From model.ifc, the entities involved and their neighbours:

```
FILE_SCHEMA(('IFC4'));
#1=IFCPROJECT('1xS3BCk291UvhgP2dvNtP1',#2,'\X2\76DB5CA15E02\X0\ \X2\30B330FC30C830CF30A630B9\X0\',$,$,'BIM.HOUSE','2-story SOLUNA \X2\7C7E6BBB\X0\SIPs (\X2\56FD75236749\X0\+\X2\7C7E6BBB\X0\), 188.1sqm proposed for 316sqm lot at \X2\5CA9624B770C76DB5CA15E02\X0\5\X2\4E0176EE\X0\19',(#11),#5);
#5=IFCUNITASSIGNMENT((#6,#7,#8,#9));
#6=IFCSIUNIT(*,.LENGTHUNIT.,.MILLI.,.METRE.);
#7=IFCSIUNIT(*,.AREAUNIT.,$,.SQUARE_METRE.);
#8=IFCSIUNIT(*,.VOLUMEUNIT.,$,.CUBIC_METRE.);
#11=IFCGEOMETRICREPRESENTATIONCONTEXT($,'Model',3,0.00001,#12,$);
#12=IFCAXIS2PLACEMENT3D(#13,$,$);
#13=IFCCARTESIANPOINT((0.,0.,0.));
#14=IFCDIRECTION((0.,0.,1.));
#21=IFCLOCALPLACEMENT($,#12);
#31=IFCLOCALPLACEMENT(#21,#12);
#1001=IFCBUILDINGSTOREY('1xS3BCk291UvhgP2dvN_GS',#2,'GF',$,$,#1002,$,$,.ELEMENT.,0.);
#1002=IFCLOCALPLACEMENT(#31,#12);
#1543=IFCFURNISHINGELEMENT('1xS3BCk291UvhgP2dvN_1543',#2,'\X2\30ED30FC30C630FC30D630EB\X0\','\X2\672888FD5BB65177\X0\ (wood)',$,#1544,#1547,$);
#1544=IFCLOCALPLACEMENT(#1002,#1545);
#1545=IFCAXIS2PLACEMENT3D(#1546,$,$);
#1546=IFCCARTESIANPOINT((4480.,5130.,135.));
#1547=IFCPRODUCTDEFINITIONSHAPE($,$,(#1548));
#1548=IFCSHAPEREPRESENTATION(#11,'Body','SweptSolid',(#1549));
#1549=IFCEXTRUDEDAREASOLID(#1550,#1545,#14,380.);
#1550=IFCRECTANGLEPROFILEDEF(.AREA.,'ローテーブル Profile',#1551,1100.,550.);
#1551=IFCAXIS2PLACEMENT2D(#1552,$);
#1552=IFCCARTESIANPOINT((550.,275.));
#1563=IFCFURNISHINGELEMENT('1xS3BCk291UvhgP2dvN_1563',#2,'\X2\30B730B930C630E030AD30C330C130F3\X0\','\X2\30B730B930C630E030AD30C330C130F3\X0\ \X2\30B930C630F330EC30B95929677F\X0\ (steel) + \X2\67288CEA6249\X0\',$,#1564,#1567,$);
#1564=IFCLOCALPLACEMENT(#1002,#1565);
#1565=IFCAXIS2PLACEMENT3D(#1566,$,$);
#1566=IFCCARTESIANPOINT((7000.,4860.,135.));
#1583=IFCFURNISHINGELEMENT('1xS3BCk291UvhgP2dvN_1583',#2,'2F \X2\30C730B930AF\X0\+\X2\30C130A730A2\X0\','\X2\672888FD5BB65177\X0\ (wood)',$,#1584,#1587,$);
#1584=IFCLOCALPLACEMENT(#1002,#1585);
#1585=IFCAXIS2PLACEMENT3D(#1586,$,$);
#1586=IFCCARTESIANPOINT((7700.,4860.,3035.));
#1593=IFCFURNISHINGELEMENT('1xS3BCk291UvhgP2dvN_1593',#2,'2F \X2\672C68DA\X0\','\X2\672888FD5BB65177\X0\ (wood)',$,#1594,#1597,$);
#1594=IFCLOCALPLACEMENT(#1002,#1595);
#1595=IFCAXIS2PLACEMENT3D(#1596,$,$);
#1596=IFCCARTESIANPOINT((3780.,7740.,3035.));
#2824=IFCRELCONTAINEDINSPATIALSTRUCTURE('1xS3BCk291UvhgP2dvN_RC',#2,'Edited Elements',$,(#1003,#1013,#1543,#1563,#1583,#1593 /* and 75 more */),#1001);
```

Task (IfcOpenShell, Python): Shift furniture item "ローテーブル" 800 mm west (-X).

```python
import ifcopenshell
import ifcopenshell.api.geometry
import ifcopenshell.util.placement

model = ifcopenshell.open("model.ifc")

item = model.by_id(1543)
matrix = ifcopenshell.util.placement.get_local_placement(item.ObjectPlacement)
matrix[0, 3] -= 800.0
ifcopenshell.api.geometry.edit_object_placement(model, product=item, matrix=matrix, is_si=False)

print(ifcopenshell.util.placement.get_local_placement(item.ObjectPlacement).round(3) + 0.0)

model.write("model_rev.ifc")
```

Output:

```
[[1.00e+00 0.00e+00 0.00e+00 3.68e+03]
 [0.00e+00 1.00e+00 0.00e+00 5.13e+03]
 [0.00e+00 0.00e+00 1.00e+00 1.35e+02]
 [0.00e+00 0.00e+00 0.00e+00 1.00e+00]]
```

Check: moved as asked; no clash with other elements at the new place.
